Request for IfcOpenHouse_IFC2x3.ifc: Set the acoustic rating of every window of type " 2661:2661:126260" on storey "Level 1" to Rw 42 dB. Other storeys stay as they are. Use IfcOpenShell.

First a look at what the model holds.

```python
import ifcopenshell
import ifcopenshell.util.element

model = ifcopenshell.open("IfcOpenHouse_IFC2x3.ifc")
print(model.schema)
storey = next(s for s in model.by_type("IfcBuildingStorey") if s.Name == "Level 1")
windows = [e for e in ifcopenshell.util.element.get_decomposition(storey) if e.is_a("IfcWindow")]
seen = {}
for e in windows:
    element_type = ifcopenshell.util.element.get_type(e)
    key = (element_type.Name if element_type != e and element_type else None, ifcopenshell.util.element.get_pset(e, "Pset_WindowCommon", "AcousticRating"))
    seen[key] = seen.get(key, 0) + 1
for (name, value), count in sorted(seen.items(), key=str):
    print(count, "x", name, "|", value)
```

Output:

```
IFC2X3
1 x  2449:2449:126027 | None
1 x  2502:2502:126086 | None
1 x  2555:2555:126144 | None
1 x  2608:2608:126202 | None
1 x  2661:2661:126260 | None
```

```python
import ifcopenshell
import ifcopenshell.api.pset
import ifcopenshell.util.element

model = ifcopenshell.open("IfcOpenHouse_IFC2x3.ifc")

storey = next(s for s in model.by_type("IfcBuildingStorey") if s.Name == "Level 1")
windows = [e for e in ifcopenshell.util.element.get_decomposition(storey) if e.is_a("IfcWindow")]

count = 0
for e in windows:
    element_type = ifcopenshell.util.element.get_type(e)
    if element_type in (None, e) or element_type.Name != " 2661:2661:126260":
        continue
    # add_pset returns the element's existing set when there is one.
    pset = ifcopenshell.api.pset.add_pset(model, product=e, name="Pset_WindowCommon")
    ifcopenshell.api.pset.edit_pset(model, pset=pset, properties={"AcousticRating": "Rw 42 dB"})
    count += 1

print(count, "windows updated")

model.write("IfcOpenHouse_IFC2x3_v2.ifc")
```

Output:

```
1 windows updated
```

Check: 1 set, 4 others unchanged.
